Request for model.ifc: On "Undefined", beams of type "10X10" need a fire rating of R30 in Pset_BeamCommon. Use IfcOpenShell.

First a look at what the model holds.

```python
import ifcopenshell
import ifcopenshell.util.element

model = ifcopenshell.open("model.ifc")
print(model.schema)
storey = next(s for s in model.by_type("IfcBuildingStorey") if s.Name == "Undefined")
beams = [e for e in ifcopenshell.util.element.get_decomposition(storey) if e.is_a("IfcBeam")]
seen = {}
for e in beams:
    element_type = ifcopenshell.util.element.get_type(e)
    key = (element_type.Name if element_type != e and element_type else None, ifcopenshell.util.element.get_pset(e, "Pset_BeamCommon", "FireRating"))
    seen[key] = seen.get(key, 0) + 1
for (name, value), count in sorted(seen.items(), key=str):
    print(count, "x", name, "|", value)
```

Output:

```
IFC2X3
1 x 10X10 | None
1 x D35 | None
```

```python
import ifcopenshell
import ifcopenshell.api.pset
import ifcopenshell.util.element

model = ifcopenshell.open("model.ifc")

storey = next(s for s in model.by_type("IfcBuildingStorey") if s.Name == "Undefined")
beams = [e for e in ifcopenshell.util.element.get_decomposition(storey) if e.is_a("IfcBeam")]

count = 0
for e in beams:
    element_type = ifcopenshell.util.element.get_type(e)
    if element_type in (None, e) or element_type.Name != "10X10":
        continue
    # add_pset returns the element's existing set when there is one.
    pset = ifcopenshell.api.pset.add_pset(model, product=e, name="Pset_BeamCommon")
    ifcopenshell.api.pset.edit_pset(model, pset=pset, properties={"FireRating": "R30"})
    count += 1

print(count, "beams updated")

model.write("model_v2.ifc")
```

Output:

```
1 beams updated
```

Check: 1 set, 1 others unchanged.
